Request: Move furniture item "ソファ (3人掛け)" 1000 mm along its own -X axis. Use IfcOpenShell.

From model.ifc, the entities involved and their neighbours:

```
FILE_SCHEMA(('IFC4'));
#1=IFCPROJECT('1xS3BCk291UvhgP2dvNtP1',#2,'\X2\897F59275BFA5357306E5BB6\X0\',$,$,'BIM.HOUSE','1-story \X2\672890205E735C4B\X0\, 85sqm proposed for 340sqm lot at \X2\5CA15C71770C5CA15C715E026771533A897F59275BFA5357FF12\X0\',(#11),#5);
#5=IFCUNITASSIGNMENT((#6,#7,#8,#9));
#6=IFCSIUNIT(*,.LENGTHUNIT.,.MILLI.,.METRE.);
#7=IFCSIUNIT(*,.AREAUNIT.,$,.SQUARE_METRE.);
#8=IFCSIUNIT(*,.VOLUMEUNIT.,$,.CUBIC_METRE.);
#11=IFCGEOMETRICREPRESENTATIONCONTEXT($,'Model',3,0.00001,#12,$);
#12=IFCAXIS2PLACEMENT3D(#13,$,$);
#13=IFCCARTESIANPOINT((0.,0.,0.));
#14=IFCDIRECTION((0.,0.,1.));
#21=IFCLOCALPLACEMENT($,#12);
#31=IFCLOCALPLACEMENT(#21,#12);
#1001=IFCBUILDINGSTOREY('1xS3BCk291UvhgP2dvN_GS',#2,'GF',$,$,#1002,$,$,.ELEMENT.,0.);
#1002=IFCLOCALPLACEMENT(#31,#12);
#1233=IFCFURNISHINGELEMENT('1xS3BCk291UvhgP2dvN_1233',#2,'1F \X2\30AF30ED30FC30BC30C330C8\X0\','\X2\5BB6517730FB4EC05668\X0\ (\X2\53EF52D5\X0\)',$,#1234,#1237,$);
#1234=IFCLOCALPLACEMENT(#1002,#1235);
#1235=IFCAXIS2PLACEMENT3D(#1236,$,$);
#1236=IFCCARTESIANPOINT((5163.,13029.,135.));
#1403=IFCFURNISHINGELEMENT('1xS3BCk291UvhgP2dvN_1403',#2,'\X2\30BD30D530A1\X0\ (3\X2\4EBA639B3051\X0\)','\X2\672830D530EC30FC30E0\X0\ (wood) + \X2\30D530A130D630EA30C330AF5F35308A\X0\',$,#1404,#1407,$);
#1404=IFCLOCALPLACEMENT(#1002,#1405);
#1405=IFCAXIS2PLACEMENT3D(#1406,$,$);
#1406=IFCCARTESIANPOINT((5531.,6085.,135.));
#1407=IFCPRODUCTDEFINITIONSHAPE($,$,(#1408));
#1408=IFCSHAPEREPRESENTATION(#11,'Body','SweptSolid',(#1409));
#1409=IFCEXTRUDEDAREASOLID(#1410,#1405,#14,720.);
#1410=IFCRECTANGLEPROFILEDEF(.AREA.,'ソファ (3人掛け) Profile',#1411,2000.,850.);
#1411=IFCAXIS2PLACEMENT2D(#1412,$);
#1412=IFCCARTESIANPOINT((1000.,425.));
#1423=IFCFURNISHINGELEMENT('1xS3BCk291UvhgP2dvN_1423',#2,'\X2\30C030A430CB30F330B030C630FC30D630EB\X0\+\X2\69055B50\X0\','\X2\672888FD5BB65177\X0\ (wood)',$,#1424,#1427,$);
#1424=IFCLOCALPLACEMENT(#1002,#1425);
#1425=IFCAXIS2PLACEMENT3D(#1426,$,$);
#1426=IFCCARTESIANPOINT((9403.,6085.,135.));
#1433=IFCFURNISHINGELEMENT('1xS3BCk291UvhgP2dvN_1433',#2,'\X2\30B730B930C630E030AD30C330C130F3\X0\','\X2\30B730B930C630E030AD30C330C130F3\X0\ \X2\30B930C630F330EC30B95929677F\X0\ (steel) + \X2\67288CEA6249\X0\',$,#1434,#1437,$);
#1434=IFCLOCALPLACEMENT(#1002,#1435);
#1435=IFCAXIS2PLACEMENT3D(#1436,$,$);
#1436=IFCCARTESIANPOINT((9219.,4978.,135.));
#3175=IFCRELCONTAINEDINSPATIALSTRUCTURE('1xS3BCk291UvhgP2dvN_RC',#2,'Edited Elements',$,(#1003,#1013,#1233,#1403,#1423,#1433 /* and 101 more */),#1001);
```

```python
import ifcopenshell
import ifcopenshell.api.geometry
import ifcopenshell.util.placement
import ifcopenshell.util.unit

model = ifcopenshell.open("model.ifc")
unit_scale = ifcopenshell.util.unit.calculate_unit_scale(model)

item = model.by_guid("1xS3BCk291UvhgP2dvN_1403")
matrix = ifcopenshell.util.placement.get_local_placement(item.ObjectPlacement)
matrix[:3, 3] -= matrix[:3, 0] * 1 / unit_scale
ifcopenshell.api.geometry.edit_object_placement(model, product=item, matrix=matrix, is_si=False)

print(ifcopenshell.util.placement.get_local_placement(item.ObjectPlacement).round(3) + 0.0)

model.write("model_rev.ifc")
```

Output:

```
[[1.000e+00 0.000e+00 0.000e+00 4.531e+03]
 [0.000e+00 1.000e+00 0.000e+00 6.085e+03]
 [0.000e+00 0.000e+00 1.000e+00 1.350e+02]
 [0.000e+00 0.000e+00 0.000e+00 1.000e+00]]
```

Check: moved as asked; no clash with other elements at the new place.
